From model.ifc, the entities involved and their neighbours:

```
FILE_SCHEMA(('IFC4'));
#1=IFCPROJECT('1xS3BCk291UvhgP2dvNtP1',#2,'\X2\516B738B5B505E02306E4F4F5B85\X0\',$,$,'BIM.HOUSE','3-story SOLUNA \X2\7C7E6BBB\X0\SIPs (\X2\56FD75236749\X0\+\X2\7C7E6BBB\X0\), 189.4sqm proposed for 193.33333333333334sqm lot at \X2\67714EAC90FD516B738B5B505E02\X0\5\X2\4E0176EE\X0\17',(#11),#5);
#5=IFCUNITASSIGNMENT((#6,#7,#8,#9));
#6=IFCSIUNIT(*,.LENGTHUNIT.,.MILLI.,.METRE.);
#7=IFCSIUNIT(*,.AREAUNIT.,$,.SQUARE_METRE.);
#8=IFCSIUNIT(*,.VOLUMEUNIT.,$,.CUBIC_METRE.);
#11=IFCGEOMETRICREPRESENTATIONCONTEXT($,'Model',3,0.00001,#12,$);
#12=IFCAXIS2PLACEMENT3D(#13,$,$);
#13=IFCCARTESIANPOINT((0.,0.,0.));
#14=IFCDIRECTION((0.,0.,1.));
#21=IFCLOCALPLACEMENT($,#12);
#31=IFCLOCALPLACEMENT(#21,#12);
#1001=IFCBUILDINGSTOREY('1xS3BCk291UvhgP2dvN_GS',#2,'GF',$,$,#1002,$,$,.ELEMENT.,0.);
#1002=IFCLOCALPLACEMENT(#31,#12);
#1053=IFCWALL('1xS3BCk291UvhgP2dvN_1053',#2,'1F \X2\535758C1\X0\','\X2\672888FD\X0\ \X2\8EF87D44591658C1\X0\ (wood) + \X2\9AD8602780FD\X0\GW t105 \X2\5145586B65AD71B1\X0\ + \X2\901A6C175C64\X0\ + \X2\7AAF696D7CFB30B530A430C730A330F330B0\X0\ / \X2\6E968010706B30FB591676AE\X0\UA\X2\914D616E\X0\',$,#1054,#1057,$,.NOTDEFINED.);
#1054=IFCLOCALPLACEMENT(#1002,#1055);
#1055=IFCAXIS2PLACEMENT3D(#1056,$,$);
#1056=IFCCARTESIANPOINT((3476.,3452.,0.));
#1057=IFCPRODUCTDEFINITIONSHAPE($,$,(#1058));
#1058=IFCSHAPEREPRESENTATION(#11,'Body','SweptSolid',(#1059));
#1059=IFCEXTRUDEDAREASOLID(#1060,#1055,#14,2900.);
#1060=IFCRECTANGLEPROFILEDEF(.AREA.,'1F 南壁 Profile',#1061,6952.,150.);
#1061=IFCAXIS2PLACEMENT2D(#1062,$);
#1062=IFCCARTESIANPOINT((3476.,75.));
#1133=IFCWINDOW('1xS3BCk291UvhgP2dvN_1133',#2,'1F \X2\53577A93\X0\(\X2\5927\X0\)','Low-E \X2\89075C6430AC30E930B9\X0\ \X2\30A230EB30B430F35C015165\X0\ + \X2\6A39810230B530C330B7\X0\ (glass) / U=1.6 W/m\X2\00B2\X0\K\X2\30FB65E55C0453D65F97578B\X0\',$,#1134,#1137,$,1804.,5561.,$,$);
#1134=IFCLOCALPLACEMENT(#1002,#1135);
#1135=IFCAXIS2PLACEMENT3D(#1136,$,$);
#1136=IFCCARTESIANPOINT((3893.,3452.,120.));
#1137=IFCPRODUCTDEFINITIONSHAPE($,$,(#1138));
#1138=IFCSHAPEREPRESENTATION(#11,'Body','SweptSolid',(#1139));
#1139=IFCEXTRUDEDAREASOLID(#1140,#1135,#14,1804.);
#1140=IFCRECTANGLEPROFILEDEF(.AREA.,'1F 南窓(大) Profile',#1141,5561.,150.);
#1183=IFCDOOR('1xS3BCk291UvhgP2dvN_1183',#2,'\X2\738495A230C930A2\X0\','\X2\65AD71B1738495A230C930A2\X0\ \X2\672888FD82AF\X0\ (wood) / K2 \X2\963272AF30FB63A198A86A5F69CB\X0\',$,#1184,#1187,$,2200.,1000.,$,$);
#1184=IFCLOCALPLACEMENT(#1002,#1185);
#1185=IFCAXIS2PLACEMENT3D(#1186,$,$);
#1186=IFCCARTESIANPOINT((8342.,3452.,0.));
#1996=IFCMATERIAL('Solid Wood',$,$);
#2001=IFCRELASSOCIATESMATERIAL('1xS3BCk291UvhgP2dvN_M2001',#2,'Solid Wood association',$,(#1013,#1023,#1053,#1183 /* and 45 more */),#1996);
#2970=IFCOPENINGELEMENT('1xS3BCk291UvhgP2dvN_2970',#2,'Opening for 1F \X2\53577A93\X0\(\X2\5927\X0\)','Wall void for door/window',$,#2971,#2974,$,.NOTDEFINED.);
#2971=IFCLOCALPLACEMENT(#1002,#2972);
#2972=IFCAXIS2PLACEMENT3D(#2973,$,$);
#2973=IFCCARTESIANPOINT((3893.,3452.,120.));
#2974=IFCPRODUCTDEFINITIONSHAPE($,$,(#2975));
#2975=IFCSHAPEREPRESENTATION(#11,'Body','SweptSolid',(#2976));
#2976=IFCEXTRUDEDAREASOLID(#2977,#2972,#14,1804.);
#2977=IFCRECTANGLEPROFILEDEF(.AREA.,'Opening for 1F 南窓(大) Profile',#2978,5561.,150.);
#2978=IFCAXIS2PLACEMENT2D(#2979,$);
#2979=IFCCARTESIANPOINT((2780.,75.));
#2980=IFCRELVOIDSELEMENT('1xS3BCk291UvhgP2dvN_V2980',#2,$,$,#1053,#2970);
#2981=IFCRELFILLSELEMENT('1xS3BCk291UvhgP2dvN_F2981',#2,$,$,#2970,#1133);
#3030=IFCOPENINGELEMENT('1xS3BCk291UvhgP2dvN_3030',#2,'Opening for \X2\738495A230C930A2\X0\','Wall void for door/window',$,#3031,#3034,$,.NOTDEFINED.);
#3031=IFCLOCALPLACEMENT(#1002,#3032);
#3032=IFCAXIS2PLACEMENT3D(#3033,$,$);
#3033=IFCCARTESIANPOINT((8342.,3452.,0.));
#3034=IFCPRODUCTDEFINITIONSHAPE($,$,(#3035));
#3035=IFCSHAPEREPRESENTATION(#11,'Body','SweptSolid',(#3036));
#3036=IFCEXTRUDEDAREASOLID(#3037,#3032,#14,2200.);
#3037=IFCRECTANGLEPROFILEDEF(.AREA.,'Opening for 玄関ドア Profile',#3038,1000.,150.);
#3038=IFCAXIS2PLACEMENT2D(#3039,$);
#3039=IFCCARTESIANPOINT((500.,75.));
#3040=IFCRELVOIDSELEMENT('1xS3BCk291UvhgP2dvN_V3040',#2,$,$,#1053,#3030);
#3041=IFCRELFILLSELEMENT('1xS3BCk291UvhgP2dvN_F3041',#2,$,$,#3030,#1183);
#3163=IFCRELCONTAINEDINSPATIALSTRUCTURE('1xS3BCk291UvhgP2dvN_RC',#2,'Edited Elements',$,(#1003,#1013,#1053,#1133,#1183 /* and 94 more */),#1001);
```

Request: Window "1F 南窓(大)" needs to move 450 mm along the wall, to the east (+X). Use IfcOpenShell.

```python
import ifcopenshell
import ifcopenshell.api.geometry
import ifcopenshell.util.placement
import ifcopenshell.util.unit

model = ifcopenshell.open("model.ifc")
unit_scale = ifcopenshell.util.unit.calculate_unit_scale(model)

window = model.by_guid("1xS3BCk291UvhgP2dvN_1133")
opening = window.FillsVoids[0].RelatingOpeningElement
wall = opening.VoidsElements[0].RelatingBuildingElement

wall_matrix = ifcopenshell.util.placement.get_local_placement(wall.ObjectPlacement)
shift = wall_matrix[:3, 0] * 0.45 / unit_scale
before = ifcopenshell.util.placement.get_local_placement(window.ObjectPlacement)[:3, 3].copy()

# The window is not placed relative to its opening, so move both.
for product in (opening, window):
    matrix = ifcopenshell.util.placement.get_local_placement(product.ObjectPlacement)
    matrix[:3, 3] += shift
    ifcopenshell.api.geometry.edit_object_placement(model, product=product, matrix=matrix, is_si=False)

after = ifcopenshell.util.placement.get_local_placement(window.ObjectPlacement)[:3, 3]
print("window moved by", (after - before).round(3) + 0.0)

model.write("model-out.ifc")
```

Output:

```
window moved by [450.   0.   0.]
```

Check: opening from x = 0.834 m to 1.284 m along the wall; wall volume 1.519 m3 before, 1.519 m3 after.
